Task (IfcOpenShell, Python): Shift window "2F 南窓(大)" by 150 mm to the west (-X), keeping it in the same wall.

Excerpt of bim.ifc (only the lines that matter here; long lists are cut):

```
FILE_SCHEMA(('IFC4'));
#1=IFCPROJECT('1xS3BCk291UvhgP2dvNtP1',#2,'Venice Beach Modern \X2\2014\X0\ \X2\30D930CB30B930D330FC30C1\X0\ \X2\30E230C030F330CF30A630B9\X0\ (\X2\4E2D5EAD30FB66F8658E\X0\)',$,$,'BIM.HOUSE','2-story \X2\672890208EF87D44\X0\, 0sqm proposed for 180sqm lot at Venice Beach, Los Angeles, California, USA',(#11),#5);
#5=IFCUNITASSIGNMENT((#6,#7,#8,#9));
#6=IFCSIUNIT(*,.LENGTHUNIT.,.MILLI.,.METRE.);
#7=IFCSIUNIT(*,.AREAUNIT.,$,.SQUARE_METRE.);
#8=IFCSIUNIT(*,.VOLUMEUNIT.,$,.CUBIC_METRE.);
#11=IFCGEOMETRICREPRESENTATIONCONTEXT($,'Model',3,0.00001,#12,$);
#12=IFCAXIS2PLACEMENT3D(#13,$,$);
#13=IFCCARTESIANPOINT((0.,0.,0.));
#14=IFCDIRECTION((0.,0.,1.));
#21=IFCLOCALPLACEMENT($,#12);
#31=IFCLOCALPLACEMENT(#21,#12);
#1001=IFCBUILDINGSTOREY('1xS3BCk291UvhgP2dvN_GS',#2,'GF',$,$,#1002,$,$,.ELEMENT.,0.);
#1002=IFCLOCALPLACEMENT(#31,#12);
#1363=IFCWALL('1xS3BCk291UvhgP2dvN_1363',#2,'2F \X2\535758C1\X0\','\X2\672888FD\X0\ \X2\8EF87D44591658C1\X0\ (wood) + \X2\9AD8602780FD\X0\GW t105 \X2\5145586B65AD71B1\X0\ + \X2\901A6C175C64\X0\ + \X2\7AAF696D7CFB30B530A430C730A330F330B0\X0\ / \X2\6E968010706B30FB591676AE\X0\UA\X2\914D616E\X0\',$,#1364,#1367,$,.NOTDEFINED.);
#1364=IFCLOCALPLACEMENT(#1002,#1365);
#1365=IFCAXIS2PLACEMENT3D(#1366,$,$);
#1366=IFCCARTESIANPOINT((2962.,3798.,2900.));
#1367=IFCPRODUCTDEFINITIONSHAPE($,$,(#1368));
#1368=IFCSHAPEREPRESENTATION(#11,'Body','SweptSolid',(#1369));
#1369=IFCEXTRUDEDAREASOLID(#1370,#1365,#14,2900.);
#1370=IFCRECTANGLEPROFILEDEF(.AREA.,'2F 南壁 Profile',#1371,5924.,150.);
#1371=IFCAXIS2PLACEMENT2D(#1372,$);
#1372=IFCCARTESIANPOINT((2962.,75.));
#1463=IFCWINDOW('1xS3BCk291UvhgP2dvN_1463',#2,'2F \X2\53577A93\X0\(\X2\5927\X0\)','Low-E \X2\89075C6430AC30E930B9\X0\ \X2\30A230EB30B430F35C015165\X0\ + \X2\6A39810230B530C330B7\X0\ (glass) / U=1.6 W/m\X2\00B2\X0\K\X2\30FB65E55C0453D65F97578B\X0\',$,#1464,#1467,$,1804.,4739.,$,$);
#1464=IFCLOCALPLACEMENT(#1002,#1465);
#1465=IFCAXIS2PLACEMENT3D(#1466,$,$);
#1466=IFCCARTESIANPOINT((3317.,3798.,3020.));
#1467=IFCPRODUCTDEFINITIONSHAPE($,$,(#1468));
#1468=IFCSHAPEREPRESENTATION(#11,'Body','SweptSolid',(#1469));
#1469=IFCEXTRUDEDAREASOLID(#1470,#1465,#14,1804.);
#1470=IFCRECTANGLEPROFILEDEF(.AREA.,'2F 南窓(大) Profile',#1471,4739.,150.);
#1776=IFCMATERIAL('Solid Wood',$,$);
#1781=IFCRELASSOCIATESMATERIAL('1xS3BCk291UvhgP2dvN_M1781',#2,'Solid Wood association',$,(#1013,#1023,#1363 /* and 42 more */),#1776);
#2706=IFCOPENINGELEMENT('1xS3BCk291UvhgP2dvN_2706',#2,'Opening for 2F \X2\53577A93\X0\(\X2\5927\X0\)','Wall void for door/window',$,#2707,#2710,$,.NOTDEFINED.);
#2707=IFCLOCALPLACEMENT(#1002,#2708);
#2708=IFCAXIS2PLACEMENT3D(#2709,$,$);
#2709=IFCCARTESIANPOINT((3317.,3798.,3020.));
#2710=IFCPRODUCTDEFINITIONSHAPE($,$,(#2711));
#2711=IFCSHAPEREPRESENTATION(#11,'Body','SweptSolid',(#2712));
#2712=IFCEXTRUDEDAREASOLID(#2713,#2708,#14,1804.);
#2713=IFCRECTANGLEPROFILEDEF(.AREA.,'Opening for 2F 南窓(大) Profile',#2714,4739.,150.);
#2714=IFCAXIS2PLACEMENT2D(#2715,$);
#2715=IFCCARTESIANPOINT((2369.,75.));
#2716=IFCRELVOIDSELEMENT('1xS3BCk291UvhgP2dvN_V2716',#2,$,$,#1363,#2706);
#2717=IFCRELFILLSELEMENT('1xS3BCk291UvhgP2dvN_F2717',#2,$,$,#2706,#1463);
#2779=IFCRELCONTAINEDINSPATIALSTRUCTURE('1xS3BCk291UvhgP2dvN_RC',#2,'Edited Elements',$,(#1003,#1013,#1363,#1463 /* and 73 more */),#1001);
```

```python
import ifcopenshell
import ifcopenshell.api.geometry
import ifcopenshell.util.placement
import ifcopenshell.util.unit

model = ifcopenshell.open("bim.ifc")
unit_scale = ifcopenshell.util.unit.calculate_unit_scale(model)

window = model.by_id(1463)
opening = window.FillsVoids[0].RelatingOpeningElement
wall = opening.VoidsElements[0].RelatingBuildingElement

wall_matrix = ifcopenshell.util.placement.get_local_placement(wall.ObjectPlacement)
shift = wall_matrix[:3, 0] * -0.15 / unit_scale
before = ifcopenshell.util.placement.get_local_placement(window.ObjectPlacement)[:3, 3].copy()

# The window is not placed relative to its opening, so move both.
for product in (opening, window):
    matrix = ifcopenshell.util.placement.get_local_placement(product.ObjectPlacement)
    matrix[:3, 3] += shift
    ifcopenshell.api.geometry.edit_object_placement(model, product=product, matrix=matrix, is_si=False)

after = ifcopenshell.util.placement.get_local_placement(window.ObjectPlacement)[:3, 3]
print("window moved by", (after - before).round(3) + 0.0)

model.write("bim_v2.ifc")
```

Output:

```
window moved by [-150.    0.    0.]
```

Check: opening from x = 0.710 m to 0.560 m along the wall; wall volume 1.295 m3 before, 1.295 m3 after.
